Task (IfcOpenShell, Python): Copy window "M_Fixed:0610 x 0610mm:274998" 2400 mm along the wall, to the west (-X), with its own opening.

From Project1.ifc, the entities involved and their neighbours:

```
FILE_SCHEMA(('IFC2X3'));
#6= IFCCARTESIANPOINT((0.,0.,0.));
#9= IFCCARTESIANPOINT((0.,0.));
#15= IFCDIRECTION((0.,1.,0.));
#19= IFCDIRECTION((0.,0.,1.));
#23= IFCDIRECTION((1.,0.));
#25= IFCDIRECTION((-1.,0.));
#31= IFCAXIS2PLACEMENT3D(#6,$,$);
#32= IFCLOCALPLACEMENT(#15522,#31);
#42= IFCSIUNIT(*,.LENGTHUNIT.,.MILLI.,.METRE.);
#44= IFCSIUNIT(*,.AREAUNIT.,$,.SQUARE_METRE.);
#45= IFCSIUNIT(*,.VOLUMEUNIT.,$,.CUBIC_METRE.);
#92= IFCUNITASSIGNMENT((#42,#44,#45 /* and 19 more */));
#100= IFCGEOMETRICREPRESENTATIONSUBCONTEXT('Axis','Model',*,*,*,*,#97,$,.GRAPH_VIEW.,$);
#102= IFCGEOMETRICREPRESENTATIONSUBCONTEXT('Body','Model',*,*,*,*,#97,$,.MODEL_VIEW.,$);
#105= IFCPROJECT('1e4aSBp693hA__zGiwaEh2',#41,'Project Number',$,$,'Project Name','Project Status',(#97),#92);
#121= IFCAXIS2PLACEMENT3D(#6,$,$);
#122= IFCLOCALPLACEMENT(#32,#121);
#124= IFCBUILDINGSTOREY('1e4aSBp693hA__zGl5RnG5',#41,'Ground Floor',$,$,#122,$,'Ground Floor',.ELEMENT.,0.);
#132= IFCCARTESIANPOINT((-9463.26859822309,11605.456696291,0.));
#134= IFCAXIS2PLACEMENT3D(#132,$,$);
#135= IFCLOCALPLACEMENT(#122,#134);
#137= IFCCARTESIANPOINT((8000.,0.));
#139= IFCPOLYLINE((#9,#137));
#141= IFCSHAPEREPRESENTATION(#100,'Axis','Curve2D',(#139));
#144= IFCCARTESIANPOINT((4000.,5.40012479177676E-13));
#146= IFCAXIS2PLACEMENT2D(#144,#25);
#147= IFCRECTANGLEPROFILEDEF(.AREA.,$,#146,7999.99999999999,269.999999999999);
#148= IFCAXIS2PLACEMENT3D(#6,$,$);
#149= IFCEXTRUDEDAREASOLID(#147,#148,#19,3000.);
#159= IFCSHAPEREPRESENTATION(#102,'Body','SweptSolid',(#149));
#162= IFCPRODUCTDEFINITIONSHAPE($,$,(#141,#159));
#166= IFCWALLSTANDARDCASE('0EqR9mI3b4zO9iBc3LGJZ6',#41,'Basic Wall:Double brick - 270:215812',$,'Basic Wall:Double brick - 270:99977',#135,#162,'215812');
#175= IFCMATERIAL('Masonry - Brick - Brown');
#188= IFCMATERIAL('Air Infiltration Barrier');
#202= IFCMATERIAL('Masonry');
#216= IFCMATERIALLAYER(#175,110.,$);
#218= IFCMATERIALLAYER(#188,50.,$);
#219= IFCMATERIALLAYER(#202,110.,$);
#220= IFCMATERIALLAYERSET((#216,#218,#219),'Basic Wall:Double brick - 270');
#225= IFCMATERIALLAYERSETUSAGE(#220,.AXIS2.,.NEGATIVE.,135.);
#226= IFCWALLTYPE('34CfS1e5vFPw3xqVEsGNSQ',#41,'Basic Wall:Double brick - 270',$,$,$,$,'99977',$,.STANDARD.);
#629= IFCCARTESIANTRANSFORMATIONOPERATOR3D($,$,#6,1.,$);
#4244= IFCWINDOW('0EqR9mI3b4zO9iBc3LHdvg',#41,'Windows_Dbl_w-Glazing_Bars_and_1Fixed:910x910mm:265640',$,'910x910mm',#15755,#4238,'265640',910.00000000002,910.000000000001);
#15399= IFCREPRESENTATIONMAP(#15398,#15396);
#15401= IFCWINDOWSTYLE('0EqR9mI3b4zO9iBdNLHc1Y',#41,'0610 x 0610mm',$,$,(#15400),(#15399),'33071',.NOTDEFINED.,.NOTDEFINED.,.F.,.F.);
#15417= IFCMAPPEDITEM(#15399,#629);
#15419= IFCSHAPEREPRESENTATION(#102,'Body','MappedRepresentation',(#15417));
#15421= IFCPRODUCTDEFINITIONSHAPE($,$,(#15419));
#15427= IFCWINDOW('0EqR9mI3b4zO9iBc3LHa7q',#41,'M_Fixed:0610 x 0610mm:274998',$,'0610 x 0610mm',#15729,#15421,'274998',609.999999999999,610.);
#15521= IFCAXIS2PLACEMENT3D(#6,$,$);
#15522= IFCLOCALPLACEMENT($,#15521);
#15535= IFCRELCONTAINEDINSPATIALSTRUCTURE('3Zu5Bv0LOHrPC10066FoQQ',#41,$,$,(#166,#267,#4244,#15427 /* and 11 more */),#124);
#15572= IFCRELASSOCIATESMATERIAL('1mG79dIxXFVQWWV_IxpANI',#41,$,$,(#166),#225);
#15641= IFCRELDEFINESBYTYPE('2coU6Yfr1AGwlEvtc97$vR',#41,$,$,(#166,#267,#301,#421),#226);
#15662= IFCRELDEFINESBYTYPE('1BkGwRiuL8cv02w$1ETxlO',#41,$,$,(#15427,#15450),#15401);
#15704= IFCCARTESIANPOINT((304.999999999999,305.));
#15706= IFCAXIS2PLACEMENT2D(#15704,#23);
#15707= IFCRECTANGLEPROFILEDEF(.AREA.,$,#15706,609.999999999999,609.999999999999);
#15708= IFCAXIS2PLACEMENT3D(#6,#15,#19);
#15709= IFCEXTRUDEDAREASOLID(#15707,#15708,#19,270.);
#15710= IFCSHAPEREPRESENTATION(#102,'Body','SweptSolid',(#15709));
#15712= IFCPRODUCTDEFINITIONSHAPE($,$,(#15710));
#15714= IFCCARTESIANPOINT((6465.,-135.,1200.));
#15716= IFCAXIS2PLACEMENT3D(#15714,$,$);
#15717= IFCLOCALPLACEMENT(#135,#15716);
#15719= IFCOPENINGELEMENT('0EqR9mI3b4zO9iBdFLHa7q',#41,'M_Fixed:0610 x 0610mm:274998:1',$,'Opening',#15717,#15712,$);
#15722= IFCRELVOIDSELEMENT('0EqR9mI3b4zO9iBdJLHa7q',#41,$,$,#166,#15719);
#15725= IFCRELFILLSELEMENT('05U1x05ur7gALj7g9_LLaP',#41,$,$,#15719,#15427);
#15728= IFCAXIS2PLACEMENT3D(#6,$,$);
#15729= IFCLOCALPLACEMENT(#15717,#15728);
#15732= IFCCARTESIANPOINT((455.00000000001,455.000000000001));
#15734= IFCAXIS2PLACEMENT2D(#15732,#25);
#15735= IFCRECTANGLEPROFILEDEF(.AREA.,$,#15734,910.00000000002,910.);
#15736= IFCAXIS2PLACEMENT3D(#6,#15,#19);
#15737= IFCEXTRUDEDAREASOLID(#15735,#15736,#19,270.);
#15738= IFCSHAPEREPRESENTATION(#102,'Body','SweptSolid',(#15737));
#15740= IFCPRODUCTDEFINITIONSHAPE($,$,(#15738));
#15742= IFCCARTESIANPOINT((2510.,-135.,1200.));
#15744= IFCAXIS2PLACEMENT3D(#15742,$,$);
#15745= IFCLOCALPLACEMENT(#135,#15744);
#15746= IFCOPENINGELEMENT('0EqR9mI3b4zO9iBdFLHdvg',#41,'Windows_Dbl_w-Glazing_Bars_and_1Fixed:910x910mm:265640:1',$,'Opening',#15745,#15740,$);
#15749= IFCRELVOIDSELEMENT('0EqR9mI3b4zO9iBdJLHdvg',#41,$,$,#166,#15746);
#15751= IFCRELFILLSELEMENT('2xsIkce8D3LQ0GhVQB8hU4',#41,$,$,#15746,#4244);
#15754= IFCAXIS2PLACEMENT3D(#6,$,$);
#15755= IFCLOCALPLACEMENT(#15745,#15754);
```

```python
import ifcopenshell
import ifcopenshell.api.feature
import ifcopenshell.api.geometry
import ifcopenshell.api.root
import ifcopenshell.geom
import ifcopenshell.util.element
import ifcopenshell.util.placement
import ifcopenshell.util.shape

model = ifcopenshell.open("Project1.ifc")
settings = ifcopenshell.geom.settings()


def volume(element):
    """Net volume in cubic metres, openings subtracted."""
    shape = ifcopenshell.geom.create_shape(settings, element)
    return ifcopenshell.util.shape.get_volume(shape.geometry)


def reuse_history(source, copy):
    """copy_class also copies each property set's owner history, people and application; keep the originals."""
    for rel in copy.IsDefinedBy:
        if rel.is_a("IfcRelDefinesByProperties") and (history := rel.RelatingPropertyDefinition.OwnerHistory):
            rel.RelatingPropertyDefinition.OwnerHistory = source.OwnerHistory
            ifcopenshell.util.element.remove_deep2(model, history)


window = model.by_id(15427)
opening = window.FillsVoids[0].RelatingOpeningElement
wall = opening.VoidsElements[0].RelatingBuildingElement
before = volume(wall)
shift = ifcopenshell.util.placement.get_local_placement(wall.ObjectPlacement)[:3, 0] * -2400.0

# copy_class copies the void relationship, type, container and properties, but no geometry.
new_opening = ifcopenshell.api.root.copy_class(model, product=opening)
new_opening.Representation = ifcopenshell.util.element.copy_deep(
    model, opening.Representation, exclude=["IfcGeometricRepresentationContext", "IfcRepresentationMap"]
)
new_opening.Name = "M_Fixed:0610 x 0610mm"
new_window = ifcopenshell.api.root.copy_class(model, product=window)
new_window.Representation = ifcopenshell.util.element.copy_deep(
    model, window.Representation, exclude=["IfcGeometricRepresentationContext", "IfcRepresentationMap"]
)
new_window.Name = "M_Fixed:0610 x 0610mm"
new_window.Tag = None
reuse_history(window, new_window)
fills = ifcopenshell.api.feature.add_filling(model, opening=new_opening, element=new_window)
fills.OwnerHistory = new_window.OwnerHistory  # required in IFC2X3

for old, new in ((opening, new_opening), (window, new_window)):
    matrix = ifcopenshell.util.placement.get_local_placement(old.ObjectPlacement)
    matrix[:3, 3] += shift
    ifcopenshell.api.geometry.edit_object_placement(model, product=new, matrix=matrix, is_si=False)

after = volume(wall)

print(f"wall volume {before:.3f} -> {after:.3f} m3")

model.write("Project1_edited.ifc")
```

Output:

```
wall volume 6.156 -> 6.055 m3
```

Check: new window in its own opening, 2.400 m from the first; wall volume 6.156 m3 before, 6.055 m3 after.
